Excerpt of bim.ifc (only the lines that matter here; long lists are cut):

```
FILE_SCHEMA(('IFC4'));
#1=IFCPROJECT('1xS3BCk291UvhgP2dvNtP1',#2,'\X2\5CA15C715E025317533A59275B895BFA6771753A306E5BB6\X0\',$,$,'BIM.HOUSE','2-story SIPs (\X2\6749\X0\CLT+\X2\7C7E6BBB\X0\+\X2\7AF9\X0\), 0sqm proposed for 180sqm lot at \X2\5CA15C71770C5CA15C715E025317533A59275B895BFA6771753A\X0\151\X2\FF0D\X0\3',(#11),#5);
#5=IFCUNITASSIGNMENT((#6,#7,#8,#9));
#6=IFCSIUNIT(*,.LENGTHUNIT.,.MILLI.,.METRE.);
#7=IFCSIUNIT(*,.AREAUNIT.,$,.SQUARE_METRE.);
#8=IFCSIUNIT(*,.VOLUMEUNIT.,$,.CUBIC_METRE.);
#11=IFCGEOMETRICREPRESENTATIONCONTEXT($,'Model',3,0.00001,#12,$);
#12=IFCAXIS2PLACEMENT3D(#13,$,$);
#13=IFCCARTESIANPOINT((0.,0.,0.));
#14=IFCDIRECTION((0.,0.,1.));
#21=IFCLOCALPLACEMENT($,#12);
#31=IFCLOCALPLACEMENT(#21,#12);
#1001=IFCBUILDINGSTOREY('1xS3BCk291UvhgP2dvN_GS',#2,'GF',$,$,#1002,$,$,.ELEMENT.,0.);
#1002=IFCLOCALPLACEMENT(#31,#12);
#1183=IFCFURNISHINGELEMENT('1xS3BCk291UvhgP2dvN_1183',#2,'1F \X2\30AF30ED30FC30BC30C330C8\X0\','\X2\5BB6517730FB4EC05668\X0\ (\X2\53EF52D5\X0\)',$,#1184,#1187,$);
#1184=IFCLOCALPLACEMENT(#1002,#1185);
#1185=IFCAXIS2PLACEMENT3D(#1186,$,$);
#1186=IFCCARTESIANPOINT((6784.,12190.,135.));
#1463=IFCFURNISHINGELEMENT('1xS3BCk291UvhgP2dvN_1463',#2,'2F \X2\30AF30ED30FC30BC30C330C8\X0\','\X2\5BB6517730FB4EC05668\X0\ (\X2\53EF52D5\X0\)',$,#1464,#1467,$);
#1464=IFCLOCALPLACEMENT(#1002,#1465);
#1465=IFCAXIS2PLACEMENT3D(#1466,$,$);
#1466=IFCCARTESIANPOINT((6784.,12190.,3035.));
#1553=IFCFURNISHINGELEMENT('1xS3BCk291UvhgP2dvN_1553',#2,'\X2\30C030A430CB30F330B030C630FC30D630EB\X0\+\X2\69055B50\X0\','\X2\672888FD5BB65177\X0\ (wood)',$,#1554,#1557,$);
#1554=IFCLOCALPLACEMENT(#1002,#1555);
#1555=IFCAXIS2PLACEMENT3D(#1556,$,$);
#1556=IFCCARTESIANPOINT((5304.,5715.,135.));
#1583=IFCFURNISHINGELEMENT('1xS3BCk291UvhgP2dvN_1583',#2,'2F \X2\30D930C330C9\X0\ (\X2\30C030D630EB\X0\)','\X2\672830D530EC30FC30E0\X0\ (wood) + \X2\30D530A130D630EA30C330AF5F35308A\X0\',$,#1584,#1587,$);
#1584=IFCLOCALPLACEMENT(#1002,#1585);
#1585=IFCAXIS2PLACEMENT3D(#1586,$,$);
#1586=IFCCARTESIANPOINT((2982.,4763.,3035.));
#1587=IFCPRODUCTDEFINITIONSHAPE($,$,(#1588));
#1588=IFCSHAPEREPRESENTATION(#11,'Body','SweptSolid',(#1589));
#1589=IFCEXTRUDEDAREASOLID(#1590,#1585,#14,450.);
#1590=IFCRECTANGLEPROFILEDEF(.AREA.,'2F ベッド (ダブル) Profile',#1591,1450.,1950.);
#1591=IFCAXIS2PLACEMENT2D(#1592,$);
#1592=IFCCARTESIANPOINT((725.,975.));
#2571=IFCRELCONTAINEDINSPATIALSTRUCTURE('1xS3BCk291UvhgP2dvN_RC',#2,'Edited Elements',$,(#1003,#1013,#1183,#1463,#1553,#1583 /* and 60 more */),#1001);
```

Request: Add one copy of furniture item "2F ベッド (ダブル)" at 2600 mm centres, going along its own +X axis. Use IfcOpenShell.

```python
import ifcopenshell
import ifcopenshell.api.geometry
import ifcopenshell.api.root
import ifcopenshell.util.element
import ifcopenshell.util.placement

model = ifcopenshell.open("bim.ifc")


def reuse_history(source, copy):
    """copy_class also copies each property set's owner history, people and application; keep the originals."""
    for rel in copy.IsDefinedBy:
        if rel.is_a("IfcRelDefinesByProperties") and (history := rel.RelatingPropertyDefinition.OwnerHistory):
            rel.RelatingPropertyDefinition.OwnerHistory = source.OwnerHistory
            ifcopenshell.util.element.remove_deep2(model, history)


source = model.by_guid("1xS3BCk291UvhgP2dvN_1583")
base = ifcopenshell.util.placement.get_local_placement(source.ObjectPlacement)
step = base[:3, 0] * 2600.0

for i in range(1, 2):
    copy = ifcopenshell.api.root.copy_class(model, product=source)
    copy.Representation = ifcopenshell.util.element.copy_deep(
        model, source.Representation, exclude=["IfcGeometricRepresentationContext", "IfcRepresentationMap"]
    )
    reuse_history(source, copy)
    matrix = base.copy()
    matrix[:3, 3] += i * step
    print("added at", matrix[:3, 3].round(3) + 0.0)
    ifcopenshell.api.geometry.edit_object_placement(model, product=copy, matrix=matrix, is_si=False)

model.write("bim_rev.ifc")
```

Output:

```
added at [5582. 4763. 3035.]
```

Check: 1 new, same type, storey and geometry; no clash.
